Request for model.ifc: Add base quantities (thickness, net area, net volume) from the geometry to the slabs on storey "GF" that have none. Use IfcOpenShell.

First a look at what the model holds.

```python
import ifcopenshell
import ifcopenshell.util.element
import ifcopenshell.util.unit

model = ifcopenshell.open("model.ifc")
print(model.schema)
for unit_type in ("LENGTHUNIT", "AREAUNIT", "VOLUMEUNIT"):
    print(unit_type, ifcopenshell.util.unit.calculate_unit_scale(model, unit_type))
storey = next(s for s in model.by_type("IfcBuildingStorey") if s.Name == "GF")
slabs = [e for e in ifcopenshell.util.element.get_decomposition(storey) if e.is_a("IfcSlab")]
for e in sorted(slabs, key=lambda e: e.id()):
    print(e.id(), e.is_a(), e.Name, list(ifcopenshell.util.element.get_psets(e, qtos_only=True)), sep=" | ")
```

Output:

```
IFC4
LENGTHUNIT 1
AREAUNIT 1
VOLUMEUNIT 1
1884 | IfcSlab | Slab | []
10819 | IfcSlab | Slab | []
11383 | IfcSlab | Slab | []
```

```python
import ifcopenshell
import ifcopenshell.api.pset
import ifcopenshell.geom
import ifcopenshell.util.element
import ifcopenshell.util.shape
import ifcopenshell.util.unit

model = ifcopenshell.open("model.ifc")
unit_scale = ifcopenshell.util.unit.calculate_unit_scale(model)
area_scale = ifcopenshell.util.unit.calculate_unit_scale(model, "AREAUNIT")
volume_scale = ifcopenshell.util.unit.calculate_unit_scale(model, "VOLUMEUNIT")
settings = ifcopenshell.geom.settings()

storey = next(s for s in model.by_type("IfcBuildingStorey") if s.Name == "GF")
slabs = [e for e in ifcopenshell.util.element.get_decomposition(storey) if e.is_a("IfcSlab")]

for e in sorted(slabs, key=lambda e: e.id()):
    if ifcopenshell.util.element.get_psets(e, qtos_only=True, should_inherit=False):
        continue
    # Geometry comes back in metres, in the element's own axes.
    shape = ifcopenshell.geom.create_shape(settings, e)
    values = {
        "Width": ifcopenshell.util.shape.get_z(shape.geometry) / unit_scale,
        "NetArea": ifcopenshell.util.shape.get_footprint_area(shape.geometry) / area_scale,
        "NetVolume": ifcopenshell.util.shape.get_volume(shape.geometry) / volume_scale,
    }
    qto = ifcopenshell.api.pset.add_qto(model, product=e, name="Qto_SlabBaseQuantities")
    ifcopenshell.api.pset.edit_qto(model, qto=qto, properties=values)
    print(e.id(), {k: round(v, 3) for k, v in values.items()})

model.write("model_edited.ifc")
```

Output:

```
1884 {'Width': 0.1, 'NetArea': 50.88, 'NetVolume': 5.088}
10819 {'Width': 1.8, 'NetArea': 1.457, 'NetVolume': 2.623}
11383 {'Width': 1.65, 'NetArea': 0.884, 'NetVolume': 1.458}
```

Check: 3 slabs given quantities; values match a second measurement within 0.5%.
